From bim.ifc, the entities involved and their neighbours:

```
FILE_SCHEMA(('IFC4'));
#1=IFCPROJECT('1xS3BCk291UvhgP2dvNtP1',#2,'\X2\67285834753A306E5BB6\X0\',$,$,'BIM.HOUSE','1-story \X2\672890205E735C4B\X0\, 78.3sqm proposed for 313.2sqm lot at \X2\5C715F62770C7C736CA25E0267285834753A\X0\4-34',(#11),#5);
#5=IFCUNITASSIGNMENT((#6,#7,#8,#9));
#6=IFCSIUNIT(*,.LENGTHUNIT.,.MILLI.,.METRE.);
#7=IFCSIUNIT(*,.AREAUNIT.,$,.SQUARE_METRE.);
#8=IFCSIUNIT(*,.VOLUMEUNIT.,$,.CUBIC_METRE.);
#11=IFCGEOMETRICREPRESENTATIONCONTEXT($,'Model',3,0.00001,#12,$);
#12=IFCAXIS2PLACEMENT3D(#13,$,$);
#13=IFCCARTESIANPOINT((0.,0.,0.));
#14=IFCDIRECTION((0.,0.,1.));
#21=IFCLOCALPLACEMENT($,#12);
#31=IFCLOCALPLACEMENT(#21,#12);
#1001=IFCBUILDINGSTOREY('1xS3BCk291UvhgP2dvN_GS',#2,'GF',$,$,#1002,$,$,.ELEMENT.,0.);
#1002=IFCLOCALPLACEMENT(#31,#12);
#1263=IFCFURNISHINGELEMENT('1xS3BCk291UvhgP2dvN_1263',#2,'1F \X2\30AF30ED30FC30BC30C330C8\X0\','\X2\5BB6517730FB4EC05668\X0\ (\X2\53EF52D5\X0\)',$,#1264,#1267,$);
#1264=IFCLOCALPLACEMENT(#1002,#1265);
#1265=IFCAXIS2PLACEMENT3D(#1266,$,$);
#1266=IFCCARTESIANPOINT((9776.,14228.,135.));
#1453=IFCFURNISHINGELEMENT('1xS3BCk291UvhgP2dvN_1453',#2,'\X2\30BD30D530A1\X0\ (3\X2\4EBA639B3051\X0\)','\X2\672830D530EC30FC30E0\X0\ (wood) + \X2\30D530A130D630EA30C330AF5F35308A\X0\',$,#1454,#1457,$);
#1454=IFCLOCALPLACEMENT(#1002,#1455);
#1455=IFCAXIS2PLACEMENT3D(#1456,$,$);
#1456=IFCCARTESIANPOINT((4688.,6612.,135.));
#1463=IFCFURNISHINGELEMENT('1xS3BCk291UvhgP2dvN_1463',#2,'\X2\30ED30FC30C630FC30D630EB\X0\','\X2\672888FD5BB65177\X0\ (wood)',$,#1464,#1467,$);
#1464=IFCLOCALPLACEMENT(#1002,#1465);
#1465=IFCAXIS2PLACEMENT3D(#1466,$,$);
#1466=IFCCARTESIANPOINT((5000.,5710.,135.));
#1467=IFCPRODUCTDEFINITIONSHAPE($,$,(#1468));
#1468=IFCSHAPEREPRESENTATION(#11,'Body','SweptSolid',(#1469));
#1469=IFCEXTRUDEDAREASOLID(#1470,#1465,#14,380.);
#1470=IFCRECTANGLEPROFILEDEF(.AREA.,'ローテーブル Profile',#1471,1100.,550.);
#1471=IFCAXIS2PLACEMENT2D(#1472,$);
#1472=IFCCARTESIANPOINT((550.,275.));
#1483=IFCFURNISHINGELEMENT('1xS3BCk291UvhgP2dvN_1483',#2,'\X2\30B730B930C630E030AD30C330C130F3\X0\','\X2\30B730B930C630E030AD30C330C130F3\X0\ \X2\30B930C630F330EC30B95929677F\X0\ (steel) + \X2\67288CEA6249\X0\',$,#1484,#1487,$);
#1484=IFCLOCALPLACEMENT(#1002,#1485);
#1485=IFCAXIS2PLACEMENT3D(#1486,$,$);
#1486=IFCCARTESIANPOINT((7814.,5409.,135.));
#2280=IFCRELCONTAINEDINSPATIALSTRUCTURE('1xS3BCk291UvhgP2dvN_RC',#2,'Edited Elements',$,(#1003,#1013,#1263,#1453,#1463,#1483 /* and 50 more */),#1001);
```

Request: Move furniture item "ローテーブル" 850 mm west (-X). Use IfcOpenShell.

```python
import ifcopenshell
import ifcopenshell.api.geometry
import ifcopenshell.util.placement

model = ifcopenshell.open("bim.ifc")

item = model.by_guid("1xS3BCk291UvhgP2dvN_1463")
matrix = ifcopenshell.util.placement.get_local_placement(item.ObjectPlacement)
matrix[0, 3] -= 850.0
ifcopenshell.api.geometry.edit_object_placement(model, product=item, matrix=matrix, is_si=False)

print(ifcopenshell.util.placement.get_local_placement(item.ObjectPlacement).round(3) + 0.0)

model.write("bim_updated.ifc")
```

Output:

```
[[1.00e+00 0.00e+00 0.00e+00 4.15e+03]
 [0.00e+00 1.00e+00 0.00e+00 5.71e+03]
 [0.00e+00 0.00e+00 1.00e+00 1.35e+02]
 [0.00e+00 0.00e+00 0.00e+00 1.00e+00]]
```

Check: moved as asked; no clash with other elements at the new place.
